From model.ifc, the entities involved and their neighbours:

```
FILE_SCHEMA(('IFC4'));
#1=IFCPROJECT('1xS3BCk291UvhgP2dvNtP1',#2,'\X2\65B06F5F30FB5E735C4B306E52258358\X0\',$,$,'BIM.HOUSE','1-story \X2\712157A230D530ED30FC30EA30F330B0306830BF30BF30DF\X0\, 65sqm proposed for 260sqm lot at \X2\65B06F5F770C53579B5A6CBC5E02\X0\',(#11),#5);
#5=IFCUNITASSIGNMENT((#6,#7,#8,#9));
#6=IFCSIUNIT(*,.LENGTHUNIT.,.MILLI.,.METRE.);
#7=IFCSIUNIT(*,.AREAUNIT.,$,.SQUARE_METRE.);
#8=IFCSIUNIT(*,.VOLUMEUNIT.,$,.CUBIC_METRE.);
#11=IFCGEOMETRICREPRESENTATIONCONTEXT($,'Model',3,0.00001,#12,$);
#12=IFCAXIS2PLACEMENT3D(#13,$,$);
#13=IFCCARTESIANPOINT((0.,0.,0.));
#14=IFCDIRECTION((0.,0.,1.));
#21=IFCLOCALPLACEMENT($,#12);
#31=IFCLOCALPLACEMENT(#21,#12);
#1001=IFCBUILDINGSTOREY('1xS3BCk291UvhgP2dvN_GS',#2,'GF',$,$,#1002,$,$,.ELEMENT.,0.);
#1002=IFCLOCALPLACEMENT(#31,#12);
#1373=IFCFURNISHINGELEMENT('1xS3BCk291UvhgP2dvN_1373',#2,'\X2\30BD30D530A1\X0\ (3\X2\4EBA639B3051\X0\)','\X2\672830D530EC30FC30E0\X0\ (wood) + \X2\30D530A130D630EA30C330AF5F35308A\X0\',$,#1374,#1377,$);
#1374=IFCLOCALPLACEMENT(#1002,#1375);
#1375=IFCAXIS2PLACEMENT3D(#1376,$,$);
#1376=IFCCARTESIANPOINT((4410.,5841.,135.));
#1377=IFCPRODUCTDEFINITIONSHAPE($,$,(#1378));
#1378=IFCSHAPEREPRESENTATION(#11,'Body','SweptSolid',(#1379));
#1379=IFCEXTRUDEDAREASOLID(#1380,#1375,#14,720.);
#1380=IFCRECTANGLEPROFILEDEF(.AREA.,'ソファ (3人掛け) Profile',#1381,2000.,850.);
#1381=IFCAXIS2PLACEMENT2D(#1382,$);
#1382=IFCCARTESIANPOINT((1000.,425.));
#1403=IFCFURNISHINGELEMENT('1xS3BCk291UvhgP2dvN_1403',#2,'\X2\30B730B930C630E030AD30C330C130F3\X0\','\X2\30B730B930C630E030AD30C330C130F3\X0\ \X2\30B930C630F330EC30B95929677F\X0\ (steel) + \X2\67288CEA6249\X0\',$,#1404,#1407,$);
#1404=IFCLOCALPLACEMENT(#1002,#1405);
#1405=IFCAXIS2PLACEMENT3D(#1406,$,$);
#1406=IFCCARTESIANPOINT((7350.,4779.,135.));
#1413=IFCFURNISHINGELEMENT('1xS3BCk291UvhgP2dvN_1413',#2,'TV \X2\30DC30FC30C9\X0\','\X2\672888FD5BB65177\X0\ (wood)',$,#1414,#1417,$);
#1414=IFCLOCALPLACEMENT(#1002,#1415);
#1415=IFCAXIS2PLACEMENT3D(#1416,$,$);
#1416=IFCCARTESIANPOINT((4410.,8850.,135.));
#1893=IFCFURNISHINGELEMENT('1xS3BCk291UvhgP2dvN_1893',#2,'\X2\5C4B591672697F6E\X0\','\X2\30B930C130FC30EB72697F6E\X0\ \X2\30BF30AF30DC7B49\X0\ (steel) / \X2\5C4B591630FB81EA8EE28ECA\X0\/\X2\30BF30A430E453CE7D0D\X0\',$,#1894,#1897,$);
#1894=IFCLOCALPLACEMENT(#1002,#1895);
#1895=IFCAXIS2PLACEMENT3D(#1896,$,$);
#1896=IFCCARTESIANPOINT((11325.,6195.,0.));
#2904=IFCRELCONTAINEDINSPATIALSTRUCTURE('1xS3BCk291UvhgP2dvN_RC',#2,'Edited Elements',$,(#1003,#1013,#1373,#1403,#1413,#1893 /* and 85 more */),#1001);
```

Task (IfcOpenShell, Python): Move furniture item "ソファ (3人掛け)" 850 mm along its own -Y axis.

```python
import ifcopenshell
import ifcopenshell.api.geometry
import ifcopenshell.util.placement

model = ifcopenshell.open("model.ifc")

item = model.by_id(1373)
matrix = ifcopenshell.util.placement.get_local_placement(item.ObjectPlacement)
matrix[:3, 3] -= matrix[:3, 1] * 850.0
ifcopenshell.api.geometry.edit_object_placement(model, product=item, matrix=matrix, is_si=False)

print(ifcopenshell.util.placement.get_local_placement(item.ObjectPlacement).round(3) + 0.0)

model.write("model_updated.ifc")
```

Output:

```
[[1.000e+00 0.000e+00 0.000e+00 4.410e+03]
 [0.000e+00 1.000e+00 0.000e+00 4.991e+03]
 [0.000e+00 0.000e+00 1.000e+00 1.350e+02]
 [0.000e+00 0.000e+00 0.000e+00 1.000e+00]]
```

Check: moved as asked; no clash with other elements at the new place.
